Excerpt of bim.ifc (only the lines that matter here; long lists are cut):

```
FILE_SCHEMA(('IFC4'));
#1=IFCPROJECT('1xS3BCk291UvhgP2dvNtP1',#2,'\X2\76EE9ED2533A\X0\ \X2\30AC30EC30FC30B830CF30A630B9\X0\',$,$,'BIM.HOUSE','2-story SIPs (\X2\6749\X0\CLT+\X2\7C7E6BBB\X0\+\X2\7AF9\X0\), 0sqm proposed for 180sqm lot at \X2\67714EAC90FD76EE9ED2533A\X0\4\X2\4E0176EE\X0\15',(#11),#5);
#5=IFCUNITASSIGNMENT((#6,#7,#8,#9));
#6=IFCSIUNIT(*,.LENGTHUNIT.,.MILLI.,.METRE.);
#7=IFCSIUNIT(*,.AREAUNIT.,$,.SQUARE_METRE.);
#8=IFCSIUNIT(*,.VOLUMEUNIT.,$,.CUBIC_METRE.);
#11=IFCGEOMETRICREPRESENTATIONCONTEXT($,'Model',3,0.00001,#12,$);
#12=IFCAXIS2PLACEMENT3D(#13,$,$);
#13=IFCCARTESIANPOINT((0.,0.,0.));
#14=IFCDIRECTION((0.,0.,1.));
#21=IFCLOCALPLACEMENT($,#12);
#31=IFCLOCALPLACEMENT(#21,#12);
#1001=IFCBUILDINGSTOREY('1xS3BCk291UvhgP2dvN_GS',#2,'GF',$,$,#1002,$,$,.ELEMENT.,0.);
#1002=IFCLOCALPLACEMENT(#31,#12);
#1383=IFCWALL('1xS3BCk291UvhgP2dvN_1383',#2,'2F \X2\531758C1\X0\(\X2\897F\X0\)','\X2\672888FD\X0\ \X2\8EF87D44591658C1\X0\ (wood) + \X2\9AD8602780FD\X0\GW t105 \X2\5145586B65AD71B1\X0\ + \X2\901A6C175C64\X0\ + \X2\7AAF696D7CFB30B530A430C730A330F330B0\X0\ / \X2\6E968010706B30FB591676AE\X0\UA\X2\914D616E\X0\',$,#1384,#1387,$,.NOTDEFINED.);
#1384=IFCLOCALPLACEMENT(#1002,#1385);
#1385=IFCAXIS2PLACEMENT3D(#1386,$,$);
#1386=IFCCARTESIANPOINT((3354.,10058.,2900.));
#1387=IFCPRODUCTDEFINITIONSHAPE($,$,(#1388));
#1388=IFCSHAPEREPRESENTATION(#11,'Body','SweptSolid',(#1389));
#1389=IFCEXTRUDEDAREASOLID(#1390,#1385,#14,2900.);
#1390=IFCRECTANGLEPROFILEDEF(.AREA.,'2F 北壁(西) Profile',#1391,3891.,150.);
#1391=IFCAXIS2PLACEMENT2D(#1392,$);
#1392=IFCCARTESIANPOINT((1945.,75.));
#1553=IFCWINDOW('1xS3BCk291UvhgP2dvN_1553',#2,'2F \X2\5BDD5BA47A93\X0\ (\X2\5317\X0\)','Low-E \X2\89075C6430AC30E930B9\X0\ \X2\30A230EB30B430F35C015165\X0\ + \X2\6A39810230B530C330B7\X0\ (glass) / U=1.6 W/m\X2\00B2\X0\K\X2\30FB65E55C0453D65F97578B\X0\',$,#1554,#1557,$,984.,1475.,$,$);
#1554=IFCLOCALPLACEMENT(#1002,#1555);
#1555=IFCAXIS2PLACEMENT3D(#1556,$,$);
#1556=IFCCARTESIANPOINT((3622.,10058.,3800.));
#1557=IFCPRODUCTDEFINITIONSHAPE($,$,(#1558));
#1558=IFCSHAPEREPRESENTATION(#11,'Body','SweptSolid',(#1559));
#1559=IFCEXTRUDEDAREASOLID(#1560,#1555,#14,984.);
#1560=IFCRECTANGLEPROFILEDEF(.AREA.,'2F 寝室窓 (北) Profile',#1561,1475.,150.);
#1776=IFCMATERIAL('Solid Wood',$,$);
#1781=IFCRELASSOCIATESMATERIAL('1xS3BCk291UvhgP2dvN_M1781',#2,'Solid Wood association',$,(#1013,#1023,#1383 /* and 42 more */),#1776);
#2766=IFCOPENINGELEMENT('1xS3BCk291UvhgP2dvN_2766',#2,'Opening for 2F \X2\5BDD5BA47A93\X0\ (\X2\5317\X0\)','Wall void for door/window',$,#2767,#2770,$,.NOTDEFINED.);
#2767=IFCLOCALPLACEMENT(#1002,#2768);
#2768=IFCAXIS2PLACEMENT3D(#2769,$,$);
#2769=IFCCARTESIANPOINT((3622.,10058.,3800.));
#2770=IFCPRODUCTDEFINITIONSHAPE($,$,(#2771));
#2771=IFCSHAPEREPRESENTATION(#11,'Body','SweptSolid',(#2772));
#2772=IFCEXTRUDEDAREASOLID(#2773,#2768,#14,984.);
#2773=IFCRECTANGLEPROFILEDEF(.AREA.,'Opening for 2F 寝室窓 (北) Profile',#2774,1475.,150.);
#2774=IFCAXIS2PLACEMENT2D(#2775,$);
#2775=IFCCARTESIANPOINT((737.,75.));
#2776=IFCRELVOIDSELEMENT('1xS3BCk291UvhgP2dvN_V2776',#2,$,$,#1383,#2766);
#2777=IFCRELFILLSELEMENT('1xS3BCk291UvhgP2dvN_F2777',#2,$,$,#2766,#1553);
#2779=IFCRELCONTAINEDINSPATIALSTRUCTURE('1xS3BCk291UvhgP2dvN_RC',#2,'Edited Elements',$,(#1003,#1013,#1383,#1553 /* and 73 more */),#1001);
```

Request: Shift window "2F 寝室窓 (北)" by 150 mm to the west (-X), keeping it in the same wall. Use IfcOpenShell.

```python
import ifcopenshell
import ifcopenshell.api.geometry
import ifcopenshell.util.placement
import ifcopenshell.util.unit

model = ifcopenshell.open("bim.ifc")
unit_scale = ifcopenshell.util.unit.calculate_unit_scale(model)

window = model.by_guid("1xS3BCk291UvhgP2dvN_1553")
opening = window.FillsVoids[0].RelatingOpeningElement
wall = opening.VoidsElements[0].RelatingBuildingElement

wall_matrix = ifcopenshell.util.placement.get_local_placement(wall.ObjectPlacement)
shift = wall_matrix[:3, 0] * -0.15 / unit_scale
before = ifcopenshell.util.placement.get_local_placement(window.ObjectPlacement)[:3, 3].copy()

# The window is not placed relative to its opening, so move both.
for product in (opening, window):
    matrix = ifcopenshell.util.placement.get_local_placement(product.ObjectPlacement)
    matrix[:3, 3] += shift
    ifcopenshell.api.geometry.edit_object_placement(model, product=product, matrix=matrix, is_si=False)

after = ifcopenshell.util.placement.get_local_placement(window.ObjectPlacement)[:3, 3]
print("window moved by", (after - before).round(3) + 0.0)

model.write("bim_edited.ifc")
```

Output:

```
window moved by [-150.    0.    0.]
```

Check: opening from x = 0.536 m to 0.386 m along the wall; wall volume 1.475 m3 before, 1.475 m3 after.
